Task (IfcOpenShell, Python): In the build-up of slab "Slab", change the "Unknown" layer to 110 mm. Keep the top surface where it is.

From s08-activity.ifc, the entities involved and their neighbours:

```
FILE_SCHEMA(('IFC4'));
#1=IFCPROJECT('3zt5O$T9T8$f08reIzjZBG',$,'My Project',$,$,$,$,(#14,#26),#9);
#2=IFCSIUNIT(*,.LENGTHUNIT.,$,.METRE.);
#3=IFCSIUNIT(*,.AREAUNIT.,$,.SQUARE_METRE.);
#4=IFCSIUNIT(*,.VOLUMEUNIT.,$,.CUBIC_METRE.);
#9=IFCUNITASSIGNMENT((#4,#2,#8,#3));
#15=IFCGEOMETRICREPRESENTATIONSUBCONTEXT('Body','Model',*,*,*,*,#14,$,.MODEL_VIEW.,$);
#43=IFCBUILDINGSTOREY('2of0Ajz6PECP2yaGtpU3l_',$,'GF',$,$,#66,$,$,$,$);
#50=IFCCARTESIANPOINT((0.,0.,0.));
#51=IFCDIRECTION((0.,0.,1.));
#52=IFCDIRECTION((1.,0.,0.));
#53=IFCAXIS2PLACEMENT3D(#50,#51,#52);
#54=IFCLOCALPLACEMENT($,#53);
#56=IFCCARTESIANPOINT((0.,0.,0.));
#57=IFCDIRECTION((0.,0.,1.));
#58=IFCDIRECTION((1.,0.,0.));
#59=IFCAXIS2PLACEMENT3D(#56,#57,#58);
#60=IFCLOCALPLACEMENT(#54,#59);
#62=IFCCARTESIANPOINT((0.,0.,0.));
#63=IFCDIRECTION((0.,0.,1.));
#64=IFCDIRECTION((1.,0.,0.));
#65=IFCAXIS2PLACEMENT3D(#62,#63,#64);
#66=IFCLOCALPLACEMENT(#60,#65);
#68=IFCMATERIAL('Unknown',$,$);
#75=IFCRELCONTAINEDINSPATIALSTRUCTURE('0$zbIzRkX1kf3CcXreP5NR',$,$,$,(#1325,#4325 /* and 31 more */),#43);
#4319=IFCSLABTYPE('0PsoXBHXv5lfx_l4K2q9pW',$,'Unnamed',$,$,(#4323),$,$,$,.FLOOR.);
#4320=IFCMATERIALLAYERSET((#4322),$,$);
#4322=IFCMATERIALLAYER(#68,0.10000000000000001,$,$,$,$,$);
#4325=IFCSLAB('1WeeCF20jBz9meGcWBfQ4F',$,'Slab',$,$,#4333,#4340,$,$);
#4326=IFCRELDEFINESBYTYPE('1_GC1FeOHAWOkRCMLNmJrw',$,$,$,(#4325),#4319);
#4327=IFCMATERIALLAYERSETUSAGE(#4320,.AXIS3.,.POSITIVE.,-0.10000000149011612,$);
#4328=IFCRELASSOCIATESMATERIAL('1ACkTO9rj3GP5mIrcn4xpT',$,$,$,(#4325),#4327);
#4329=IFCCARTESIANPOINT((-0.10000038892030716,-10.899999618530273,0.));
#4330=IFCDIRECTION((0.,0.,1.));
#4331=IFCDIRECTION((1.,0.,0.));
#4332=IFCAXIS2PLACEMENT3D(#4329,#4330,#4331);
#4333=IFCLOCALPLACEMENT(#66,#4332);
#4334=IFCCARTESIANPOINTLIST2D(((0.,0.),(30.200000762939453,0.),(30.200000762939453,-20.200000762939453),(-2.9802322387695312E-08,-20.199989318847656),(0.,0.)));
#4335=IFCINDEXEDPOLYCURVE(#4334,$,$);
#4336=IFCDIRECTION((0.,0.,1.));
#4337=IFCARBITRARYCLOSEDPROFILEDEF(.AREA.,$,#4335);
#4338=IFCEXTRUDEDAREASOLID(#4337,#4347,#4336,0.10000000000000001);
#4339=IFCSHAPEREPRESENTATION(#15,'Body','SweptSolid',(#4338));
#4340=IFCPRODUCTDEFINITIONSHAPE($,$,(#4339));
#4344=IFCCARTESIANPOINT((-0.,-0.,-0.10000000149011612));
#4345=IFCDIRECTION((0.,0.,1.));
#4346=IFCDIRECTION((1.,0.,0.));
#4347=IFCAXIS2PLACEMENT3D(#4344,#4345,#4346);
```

```python
import ifcopenshell
import ifcopenshell.util.element
import ifcopenshell.util.representation
import ifcopenshell.util.unit

model = ifcopenshell.open("s08-activity.ifc")
unit_scale = ifcopenshell.util.unit.calculate_unit_scale(model)

layer_set = model.by_id(4320)
layer = next(l for l in layer_set.MaterialLayers if l.Material and l.Material.Name == "Unknown")
change = 0.11 / unit_scale - layer.LayerThickness
layer.LayerThickness += change

# Geometry does not follow the layer set by itself.
slabs = [e for e in ifcopenshell.util.element.get_elements_by_material(model, layer_set) if e.is_a("IfcSlab")]
for slab in sorted(slabs, key=lambda e: e.id()):
    body = ifcopenshell.util.representation.get_representation(slab, "Model", "Body")
    solid = body.Items[0]
    old_depth = solid.Depth
    solid.Depth += change
    # Extruded upwards: lower the start of the extrusion so the top stays.
    x, y, z = solid.Position.Location.Coordinates
    solid.Position.Location = model.createIfcCartesianPoint((x, y, z - change))
    print(slab.id(), f"{old_depth:g} -> {solid.Depth:g}")

# The layers are counted up from the underside, which has moved.
for usage in {ifcopenshell.util.element.get_material(slab) for slab in slabs}:
    usage.OffsetFromReferenceLine -= change

model.write("s08-activity_rev.ifc")
```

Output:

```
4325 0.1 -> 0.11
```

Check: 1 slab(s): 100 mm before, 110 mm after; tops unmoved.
